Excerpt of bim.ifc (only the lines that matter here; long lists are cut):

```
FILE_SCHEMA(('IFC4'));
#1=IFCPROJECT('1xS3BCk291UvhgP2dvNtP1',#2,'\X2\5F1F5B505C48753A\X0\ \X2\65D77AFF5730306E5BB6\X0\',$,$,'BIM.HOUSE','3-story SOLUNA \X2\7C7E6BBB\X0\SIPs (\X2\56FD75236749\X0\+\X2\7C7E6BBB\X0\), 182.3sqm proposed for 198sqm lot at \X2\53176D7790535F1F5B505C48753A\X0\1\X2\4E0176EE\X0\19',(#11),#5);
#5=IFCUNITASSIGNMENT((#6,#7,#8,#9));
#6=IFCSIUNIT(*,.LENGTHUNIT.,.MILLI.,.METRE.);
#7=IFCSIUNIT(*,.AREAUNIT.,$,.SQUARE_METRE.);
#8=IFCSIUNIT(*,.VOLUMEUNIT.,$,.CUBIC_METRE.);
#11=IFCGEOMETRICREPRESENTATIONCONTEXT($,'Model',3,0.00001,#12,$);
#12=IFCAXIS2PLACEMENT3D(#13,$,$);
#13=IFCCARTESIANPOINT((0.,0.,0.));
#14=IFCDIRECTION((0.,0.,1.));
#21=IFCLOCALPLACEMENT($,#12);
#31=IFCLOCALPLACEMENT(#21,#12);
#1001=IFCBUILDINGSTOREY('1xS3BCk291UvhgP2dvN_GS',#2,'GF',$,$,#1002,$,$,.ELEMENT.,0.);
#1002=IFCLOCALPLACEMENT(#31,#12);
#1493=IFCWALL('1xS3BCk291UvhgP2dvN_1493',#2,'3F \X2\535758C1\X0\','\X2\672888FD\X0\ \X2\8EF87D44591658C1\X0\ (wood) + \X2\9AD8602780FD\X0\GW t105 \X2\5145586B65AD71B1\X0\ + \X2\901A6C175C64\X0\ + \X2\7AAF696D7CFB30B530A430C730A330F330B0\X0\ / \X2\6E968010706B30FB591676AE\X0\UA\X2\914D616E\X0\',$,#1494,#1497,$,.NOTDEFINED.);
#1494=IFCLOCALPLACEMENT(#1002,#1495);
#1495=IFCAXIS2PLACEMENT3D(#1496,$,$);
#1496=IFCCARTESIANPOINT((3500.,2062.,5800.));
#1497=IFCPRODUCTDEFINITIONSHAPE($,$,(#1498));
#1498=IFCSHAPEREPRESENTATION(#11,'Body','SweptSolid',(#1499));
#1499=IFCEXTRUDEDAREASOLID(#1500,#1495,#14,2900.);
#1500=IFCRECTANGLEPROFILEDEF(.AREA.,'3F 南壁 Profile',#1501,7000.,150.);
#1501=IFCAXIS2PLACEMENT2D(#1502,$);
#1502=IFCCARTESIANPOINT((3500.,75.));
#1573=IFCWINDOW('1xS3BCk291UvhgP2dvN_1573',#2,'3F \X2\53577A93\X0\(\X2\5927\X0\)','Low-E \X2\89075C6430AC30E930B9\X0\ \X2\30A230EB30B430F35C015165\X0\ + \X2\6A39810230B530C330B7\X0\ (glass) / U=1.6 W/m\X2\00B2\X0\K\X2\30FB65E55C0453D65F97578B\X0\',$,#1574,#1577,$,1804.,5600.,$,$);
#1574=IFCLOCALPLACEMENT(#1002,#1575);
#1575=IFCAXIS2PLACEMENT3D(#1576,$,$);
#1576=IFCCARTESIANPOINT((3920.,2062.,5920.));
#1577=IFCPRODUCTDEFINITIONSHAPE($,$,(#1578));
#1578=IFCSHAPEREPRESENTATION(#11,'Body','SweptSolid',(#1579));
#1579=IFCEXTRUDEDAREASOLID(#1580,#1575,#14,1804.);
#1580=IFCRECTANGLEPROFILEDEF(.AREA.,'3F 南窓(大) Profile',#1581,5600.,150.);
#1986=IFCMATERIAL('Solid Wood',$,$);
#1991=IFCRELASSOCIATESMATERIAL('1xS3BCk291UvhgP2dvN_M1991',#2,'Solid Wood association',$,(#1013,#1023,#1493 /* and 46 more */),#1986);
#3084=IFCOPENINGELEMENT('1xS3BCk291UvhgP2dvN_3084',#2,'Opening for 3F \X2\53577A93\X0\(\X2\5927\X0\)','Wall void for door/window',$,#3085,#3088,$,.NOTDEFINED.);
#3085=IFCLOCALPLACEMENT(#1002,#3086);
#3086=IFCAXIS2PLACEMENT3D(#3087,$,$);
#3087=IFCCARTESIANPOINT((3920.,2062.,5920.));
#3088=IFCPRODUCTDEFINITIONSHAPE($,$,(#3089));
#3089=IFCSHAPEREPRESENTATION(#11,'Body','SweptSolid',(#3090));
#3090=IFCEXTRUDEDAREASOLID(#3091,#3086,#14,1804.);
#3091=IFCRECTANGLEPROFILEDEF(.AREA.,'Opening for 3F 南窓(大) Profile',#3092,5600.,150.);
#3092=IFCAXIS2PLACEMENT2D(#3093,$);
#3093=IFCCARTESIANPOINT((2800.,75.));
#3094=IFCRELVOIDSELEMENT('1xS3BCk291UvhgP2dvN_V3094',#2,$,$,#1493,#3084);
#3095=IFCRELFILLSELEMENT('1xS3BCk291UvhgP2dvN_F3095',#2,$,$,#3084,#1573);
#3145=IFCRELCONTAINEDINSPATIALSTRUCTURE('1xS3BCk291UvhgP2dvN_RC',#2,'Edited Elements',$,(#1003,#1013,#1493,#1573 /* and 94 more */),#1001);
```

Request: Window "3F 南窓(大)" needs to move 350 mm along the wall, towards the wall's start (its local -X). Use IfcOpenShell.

```python
import ifcopenshell
import ifcopenshell.api.geometry
import ifcopenshell.util.placement

model = ifcopenshell.open("bim.ifc")

window = model.by_guid("1xS3BCk291UvhgP2dvN_1573")
opening = window.FillsVoids[0].RelatingOpeningElement
wall = opening.VoidsElements[0].RelatingBuildingElement

wall_matrix = ifcopenshell.util.placement.get_local_placement(wall.ObjectPlacement)
shift = wall_matrix[:3, 0] * -350.0
before = ifcopenshell.util.placement.get_local_placement(window.ObjectPlacement)[:3, 3].copy()

# The window is not placed relative to its opening, so move both.
for product in (opening, window):
    matrix = ifcopenshell.util.placement.get_local_placement(product.ObjectPlacement)
    matrix[:3, 3] += shift
    ifcopenshell.api.geometry.edit_object_placement(model, product=product, matrix=matrix, is_si=False)

after = ifcopenshell.util.placement.get_local_placement(window.ObjectPlacement)[:3, 3]
print("window moved by", (after - before).round(3) + 0.0)

model.write("bim-out.ifc")
```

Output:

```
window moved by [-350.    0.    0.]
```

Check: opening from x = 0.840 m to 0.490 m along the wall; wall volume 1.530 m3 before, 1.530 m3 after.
